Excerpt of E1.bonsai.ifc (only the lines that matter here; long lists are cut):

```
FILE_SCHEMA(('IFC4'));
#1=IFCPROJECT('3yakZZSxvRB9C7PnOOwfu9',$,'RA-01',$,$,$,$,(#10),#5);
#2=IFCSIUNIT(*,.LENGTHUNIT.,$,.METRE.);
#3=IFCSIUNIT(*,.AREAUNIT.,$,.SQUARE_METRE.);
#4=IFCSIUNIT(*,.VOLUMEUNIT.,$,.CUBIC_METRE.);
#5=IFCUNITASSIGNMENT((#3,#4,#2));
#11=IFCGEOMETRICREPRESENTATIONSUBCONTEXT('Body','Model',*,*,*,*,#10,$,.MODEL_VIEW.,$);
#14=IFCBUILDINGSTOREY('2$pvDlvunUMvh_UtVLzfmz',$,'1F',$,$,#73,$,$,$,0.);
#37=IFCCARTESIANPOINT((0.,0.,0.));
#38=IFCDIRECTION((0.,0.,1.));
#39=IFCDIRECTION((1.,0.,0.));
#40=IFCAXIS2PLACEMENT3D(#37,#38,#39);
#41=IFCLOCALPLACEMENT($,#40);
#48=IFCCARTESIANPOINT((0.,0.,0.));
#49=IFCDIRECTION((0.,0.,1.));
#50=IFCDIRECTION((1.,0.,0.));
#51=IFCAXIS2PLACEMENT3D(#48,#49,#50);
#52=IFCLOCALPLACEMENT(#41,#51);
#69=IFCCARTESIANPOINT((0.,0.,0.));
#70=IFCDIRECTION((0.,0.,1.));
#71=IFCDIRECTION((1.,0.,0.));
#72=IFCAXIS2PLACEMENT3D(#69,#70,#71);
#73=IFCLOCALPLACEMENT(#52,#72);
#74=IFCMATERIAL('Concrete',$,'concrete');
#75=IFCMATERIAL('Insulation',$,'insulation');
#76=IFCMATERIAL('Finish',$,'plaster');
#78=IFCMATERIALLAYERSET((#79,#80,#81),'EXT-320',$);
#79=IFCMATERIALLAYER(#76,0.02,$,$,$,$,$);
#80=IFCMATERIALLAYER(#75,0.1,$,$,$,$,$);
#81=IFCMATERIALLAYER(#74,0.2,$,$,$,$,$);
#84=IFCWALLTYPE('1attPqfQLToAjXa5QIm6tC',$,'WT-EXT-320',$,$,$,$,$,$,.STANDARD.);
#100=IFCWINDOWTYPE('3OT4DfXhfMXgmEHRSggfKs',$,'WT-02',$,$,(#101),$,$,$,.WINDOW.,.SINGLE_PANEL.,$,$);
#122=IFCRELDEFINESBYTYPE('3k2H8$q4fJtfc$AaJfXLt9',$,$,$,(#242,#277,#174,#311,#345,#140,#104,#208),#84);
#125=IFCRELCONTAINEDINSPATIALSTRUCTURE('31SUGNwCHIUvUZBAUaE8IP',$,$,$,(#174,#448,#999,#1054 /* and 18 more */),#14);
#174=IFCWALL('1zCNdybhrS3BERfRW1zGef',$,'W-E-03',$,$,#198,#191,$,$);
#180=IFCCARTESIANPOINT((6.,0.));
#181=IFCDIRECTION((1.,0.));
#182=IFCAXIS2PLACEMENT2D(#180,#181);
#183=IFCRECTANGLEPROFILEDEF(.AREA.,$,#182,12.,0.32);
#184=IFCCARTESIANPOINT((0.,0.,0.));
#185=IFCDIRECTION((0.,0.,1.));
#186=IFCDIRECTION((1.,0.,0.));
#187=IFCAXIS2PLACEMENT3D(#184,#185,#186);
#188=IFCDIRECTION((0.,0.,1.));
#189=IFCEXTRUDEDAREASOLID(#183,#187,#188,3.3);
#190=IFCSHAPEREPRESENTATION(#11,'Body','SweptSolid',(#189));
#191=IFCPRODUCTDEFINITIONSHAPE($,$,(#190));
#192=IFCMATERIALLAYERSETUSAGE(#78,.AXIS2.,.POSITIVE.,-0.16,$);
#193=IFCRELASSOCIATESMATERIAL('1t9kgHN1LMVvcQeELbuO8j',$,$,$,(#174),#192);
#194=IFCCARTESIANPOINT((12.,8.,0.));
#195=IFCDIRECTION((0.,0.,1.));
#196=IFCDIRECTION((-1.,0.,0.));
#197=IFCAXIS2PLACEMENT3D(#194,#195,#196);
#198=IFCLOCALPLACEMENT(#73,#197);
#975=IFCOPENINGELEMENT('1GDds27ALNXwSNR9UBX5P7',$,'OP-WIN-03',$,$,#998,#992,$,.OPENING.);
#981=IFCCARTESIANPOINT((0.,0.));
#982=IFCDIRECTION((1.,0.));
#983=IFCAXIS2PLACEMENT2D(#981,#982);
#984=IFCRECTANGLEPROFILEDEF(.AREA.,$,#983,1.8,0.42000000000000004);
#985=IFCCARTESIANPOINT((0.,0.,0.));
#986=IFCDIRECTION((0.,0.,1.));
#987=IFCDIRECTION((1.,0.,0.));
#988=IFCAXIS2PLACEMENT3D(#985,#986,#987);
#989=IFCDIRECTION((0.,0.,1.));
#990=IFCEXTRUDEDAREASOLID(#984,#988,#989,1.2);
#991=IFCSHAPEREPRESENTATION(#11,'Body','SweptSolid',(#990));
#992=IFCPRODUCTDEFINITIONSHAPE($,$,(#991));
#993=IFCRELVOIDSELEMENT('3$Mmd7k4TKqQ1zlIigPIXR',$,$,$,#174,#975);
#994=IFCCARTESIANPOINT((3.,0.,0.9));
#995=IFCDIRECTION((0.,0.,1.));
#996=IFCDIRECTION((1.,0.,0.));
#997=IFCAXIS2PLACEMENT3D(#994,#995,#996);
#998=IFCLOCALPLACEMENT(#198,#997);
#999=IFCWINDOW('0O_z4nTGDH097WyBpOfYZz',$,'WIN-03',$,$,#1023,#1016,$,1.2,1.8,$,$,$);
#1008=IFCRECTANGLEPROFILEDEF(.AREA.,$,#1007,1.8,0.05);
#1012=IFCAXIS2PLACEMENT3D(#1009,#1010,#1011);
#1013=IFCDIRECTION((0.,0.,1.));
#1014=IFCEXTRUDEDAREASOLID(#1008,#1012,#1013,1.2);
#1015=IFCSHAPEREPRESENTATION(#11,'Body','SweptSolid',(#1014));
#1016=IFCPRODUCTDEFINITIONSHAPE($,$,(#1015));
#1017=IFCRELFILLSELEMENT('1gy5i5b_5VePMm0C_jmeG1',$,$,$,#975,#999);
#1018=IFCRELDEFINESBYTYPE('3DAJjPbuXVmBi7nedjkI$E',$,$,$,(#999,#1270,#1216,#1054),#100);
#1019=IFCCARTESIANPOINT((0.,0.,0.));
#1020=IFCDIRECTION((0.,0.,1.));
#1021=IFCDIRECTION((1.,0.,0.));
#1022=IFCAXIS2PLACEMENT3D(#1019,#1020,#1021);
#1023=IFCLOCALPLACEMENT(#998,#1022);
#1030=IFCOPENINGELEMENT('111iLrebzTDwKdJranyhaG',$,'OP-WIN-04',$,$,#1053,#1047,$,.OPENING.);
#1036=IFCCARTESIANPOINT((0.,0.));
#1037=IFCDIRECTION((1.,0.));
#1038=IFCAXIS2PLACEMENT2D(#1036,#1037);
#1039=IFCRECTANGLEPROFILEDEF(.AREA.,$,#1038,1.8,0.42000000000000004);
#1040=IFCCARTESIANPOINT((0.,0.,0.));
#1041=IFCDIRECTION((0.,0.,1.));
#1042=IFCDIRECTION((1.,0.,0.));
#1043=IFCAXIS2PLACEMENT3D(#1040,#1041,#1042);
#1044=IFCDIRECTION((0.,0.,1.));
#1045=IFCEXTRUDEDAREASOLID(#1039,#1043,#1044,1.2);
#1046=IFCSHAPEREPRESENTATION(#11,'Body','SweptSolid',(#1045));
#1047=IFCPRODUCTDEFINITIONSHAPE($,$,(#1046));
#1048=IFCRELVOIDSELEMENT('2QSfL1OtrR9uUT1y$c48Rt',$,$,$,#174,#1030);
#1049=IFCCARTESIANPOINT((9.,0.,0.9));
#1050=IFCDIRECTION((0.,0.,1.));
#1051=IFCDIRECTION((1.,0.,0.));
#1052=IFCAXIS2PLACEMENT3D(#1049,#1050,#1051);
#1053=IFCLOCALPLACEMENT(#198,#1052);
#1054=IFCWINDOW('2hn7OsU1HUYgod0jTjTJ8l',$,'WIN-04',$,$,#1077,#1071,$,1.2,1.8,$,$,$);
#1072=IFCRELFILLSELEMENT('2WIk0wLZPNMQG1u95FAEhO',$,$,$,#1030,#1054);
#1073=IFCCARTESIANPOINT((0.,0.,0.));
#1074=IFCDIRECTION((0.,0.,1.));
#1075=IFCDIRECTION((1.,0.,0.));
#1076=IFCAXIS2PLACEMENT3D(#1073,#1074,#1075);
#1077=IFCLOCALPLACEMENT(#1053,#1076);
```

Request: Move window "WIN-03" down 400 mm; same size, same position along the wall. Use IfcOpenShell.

```python
import numpy as np
import ifcopenshell
import ifcopenshell.api.geometry
import ifcopenshell.util.placement
import ifcopenshell.util.unit

model = ifcopenshell.open("E1.bonsai.ifc")
unit_scale = ifcopenshell.util.unit.calculate_unit_scale(model)

window = model.by_guid("0O_z4nTGDH097WyBpOfYZz")
opening = window.FillsVoids[0].RelatingOpeningElement
dz = -0.4 / unit_scale

shift = np.array([0.0, 0.0, dz])
# The window is placed relative to its opening, so it follows when the opening moves.
matrix = ifcopenshell.util.placement.get_local_placement(opening.ObjectPlacement)
matrix[:3, 3] += shift
ifcopenshell.api.geometry.edit_object_placement(
    model, product=opening, matrix=matrix, is_si=False, should_transform_children=True
)

print(f"moved by {dz * unit_scale:+.3f} m")

model.write("E1.bonsai-out.ifc")
```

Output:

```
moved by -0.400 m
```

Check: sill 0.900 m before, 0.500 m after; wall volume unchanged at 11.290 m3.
